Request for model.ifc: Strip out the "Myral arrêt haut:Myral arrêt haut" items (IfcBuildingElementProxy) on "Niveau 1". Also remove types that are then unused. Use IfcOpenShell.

First a look at what the model holds.

```python
import ifcopenshell
import ifcopenshell.util.element

model = ifcopenshell.open("model.ifc")
print(model.schema)
storey = next(s for s in model.by_type("IfcBuildingStorey") if s.Name == "Niveau 1")
proxies = [e for e in ifcopenshell.util.element.get_decomposition(storey) if e.is_a("IfcBuildingElementProxy")]
seen = {}
for e in proxies:
    element_type = ifcopenshell.util.element.get_type(e)
    name = element_type.Name if element_type not in (None, e) else None
    seen[name] = seen.get(name, 0) + 1
for name, count in sorted(seen.items(), key=str):
    print(count, "x", name)
```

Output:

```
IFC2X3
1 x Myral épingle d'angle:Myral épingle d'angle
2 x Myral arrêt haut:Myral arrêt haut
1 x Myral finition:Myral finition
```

```python
import ifcopenshell
import ifcopenshell.api.root
import ifcopenshell.util.element

model = ifcopenshell.open("model.ifc")

storey = next(s for s in model.by_type("IfcBuildingStorey") if s.Name == "Niveau 1")
proxies = [e for e in ifcopenshell.util.element.get_decomposition(storey) if e.is_a("IfcBuildingElementProxy")]
targets = [e for e in proxies if (t := ifcopenshell.util.element.get_type(e)) not in (None, e) and t.Name == "Myral arrêt haut:Myral arrêt haut"]
types = {ifcopenshell.util.element.get_type(e) for e in targets} - {None, *targets}

for e in targets:
    ifcopenshell.api.root.remove_product(model, product=e)
print(len(targets), "removed")

unused = [t for t in types if not ifcopenshell.util.element.get_types(t)]
for t in unused:
    ifcopenshell.api.root.remove_product(model, product=t)
print(len(unused), "unused types removed")

model.write("model_v2.ifc")
```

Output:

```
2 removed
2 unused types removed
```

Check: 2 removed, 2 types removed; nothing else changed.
